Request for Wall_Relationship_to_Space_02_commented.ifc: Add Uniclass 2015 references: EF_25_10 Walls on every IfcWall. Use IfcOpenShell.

First a look at what the model holds.

```python
import ifcopenshell

model = ifcopenshell.open("Wall_Relationship_to_Space_02_commented.ifc")
print(model.schema)
print("classifications:", [c.Name for c in model.by_type("IfcClassification")])
for ifc_class in ("IfcDoor", "IfcRoof", "IfcStair", "IfcWall", "IfcWindow"):
    print(ifc_class, len(model.by_type(ifc_class)))
```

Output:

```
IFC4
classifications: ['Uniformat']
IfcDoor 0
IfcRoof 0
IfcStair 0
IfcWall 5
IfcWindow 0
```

```python
import ifcopenshell
import ifcopenshell.api.classification

model = ifcopenshell.open("Wall_Relationship_to_Space_02_commented.ifc")

system = ifcopenshell.api.classification.add_classification(model, classification="Uniclass 2015")

codes = {
    "IfcWall": ("EF_25_10", "Walls"),
}
for ifc_class, (code, name) in codes.items():
    products = model.by_type(ifc_class)
    ifcopenshell.api.classification.add_reference(
        model, products=products, classification=system, identification=code, name=name
    )
    print(code, len(products))

model.write("Wall_Relationship_to_Space_02_commented-out.ifc")
```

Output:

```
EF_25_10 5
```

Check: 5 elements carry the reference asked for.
